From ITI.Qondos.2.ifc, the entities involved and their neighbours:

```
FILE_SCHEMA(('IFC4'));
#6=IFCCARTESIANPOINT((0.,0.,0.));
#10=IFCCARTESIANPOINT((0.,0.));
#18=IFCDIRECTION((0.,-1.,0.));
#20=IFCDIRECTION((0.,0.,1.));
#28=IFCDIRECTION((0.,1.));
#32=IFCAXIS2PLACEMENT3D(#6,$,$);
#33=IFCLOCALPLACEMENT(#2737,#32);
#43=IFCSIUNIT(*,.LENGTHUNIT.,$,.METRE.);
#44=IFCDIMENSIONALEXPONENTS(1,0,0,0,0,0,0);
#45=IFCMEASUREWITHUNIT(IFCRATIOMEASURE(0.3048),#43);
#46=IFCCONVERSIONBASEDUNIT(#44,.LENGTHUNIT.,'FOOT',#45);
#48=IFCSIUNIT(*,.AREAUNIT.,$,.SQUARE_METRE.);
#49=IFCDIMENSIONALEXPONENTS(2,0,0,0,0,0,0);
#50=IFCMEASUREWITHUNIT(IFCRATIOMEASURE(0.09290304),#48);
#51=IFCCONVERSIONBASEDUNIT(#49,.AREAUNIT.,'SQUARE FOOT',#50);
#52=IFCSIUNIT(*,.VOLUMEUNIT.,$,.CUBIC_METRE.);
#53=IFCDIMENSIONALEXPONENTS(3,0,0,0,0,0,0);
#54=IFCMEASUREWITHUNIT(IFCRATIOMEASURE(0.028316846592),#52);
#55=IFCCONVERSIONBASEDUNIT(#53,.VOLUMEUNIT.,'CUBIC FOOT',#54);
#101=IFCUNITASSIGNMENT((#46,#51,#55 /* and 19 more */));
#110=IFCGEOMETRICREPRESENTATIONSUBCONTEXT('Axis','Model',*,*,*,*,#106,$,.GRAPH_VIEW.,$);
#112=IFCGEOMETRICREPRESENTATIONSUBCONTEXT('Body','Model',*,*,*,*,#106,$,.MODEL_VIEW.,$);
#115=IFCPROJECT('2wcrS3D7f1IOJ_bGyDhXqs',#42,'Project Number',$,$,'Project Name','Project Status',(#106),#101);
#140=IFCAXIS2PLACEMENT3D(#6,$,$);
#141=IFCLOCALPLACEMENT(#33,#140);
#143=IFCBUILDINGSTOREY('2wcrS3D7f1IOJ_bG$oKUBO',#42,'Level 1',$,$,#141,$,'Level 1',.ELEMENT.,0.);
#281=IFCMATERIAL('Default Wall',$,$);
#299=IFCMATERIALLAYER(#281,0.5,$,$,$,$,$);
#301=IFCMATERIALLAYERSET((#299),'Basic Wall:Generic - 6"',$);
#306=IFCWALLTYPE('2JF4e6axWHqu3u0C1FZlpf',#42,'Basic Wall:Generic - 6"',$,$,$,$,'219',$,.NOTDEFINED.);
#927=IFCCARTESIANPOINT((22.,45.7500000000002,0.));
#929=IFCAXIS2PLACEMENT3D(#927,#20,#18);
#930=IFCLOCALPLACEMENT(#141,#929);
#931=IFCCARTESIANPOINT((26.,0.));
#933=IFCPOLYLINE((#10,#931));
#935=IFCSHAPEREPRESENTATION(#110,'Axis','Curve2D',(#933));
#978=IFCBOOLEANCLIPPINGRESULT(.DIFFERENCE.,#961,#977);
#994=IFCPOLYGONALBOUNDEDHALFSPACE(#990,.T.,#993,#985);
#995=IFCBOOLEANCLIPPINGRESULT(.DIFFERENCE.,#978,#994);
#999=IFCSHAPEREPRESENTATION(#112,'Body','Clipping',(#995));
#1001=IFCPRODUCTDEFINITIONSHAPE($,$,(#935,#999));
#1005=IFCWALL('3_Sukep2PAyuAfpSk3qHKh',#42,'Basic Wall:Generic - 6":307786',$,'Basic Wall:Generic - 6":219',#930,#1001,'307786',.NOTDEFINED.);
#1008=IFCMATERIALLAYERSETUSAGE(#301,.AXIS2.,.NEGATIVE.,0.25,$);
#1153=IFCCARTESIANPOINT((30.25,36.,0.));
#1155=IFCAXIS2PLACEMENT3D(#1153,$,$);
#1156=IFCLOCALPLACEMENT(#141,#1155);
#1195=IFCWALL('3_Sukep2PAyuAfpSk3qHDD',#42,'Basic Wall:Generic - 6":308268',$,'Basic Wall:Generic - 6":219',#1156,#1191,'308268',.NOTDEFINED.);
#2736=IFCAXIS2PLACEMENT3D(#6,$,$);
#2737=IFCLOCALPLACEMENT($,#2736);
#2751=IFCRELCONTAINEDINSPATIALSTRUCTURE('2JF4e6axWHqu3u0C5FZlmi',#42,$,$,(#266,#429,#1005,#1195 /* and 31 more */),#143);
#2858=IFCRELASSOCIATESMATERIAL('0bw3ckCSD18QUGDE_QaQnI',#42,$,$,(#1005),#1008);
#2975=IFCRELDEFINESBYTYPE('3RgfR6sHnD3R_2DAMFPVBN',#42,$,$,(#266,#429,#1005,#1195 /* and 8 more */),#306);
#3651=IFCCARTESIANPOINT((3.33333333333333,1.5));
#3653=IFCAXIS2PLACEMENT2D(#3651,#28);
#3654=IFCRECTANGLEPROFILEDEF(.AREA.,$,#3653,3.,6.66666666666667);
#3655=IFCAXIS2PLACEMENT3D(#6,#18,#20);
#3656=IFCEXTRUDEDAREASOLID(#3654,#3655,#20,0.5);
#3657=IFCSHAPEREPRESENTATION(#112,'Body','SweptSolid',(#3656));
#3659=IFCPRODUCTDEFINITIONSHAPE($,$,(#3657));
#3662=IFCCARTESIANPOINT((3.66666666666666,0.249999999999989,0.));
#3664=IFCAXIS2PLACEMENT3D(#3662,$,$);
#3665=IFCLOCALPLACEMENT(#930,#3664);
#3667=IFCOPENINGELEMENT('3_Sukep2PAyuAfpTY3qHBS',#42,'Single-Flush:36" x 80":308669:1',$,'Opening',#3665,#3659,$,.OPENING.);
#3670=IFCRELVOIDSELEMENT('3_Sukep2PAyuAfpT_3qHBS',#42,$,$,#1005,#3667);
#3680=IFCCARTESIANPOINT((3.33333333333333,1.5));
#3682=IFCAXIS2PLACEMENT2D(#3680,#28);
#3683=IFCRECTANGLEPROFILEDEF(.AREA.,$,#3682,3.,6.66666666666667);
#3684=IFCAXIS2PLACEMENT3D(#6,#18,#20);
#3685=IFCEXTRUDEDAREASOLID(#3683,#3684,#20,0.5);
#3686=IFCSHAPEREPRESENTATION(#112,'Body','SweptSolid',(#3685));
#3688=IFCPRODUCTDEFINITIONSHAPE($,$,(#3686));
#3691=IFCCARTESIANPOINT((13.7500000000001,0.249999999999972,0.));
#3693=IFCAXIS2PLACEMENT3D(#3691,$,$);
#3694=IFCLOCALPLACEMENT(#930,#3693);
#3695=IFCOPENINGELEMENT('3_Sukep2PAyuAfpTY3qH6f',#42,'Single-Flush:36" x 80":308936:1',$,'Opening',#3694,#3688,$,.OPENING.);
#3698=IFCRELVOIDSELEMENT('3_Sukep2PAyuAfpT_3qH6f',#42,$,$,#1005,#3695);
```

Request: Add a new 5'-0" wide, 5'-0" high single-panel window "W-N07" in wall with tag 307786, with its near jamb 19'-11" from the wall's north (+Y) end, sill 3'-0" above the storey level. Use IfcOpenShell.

```python
import numpy as np
import ifcopenshell
import ifcopenshell.api.feature
import ifcopenshell.api.geometry
import ifcopenshell.api.root
import ifcopenshell.api.spatial
import ifcopenshell.geom
import ifcopenshell.util.element
import ifcopenshell.util.placement
import ifcopenshell.util.representation
import ifcopenshell.util.shape
import ifcopenshell.util.unit

model = ifcopenshell.open("ITI.Qondos.2.ifc")
unit_scale = ifcopenshell.util.unit.calculate_unit_scale(model)
settings = ifcopenshell.geom.settings()


def volume(element):
    """Net volume in cubic metres, openings subtracted."""
    shape = ifcopenshell.geom.create_shape(settings, element)
    return ifcopenshell.util.shape.get_volume(shape.geometry)


wall = model.by_guid("3_Sukep2PAyuAfpSk3qHKh")
storey = ifcopenshell.util.element.get_container(wall, ifc_class="IfcBuildingStorey")
context = ifcopenshell.util.representation.get_context(model, "Model", "Body", "MODEL_VIEW")
before = volume(wall)

width, height, from_end, sill = 1.524, 1.524, 6.0706, 0.9144  # metres

# The wall runs along its own X axis, and the end named is its -X end.
wall_shape = ifcopenshell.geom.create_shape(settings, wall)
x, y, z = ifcopenshell.util.shape.get_vertices(wall_shape.geometry).T
start = x.min() + from_end
face, thickness = float(y.min()), float(y.max() - y.min())
wall_matrix = ifcopenshell.util.placement.get_local_placement(wall.ObjectPlacement)
level = ifcopenshell.util.placement.get_local_placement(storey.ObjectPlacement)[2, 3]


def in_wall(x, y):
    """Placement at x, y metres in the wall's axes, at sill height."""
    matrix = wall_matrix.copy()
    matrix[:, 3] = wall_matrix @ np.array([x / unit_scale, y / unit_scale, 0.0, 1.0])
    matrix[2, 3] = level + sill / unit_scale
    return matrix


# Opening: a box that overshoots both wall faces by 50 mm.
opening = ifcopenshell.api.root.create_entity(model, ifc_class="IfcOpeningElement", predefined_type="OPENING")
box = ifcopenshell.api.geometry.add_wall_representation(
    model, context=context, length=width, height=height, thickness=thickness + 0.1
)
ifcopenshell.api.geometry.assign_representation(model, product=opening, representation=box)
ifcopenshell.api.geometry.edit_object_placement(model, product=opening, matrix=in_wall(start, face - 0.05), is_si=False)
ifcopenshell.api.feature.add_feature(model, feature=opening, element=wall)

window = ifcopenshell.api.root.create_entity(model, ifc_class="IfcWindow", name="W-N07", predefined_type="WINDOW")
window.OverallWidth, window.OverallHeight = width / unit_scale, height / unit_scale
window.PartitioningType = "SINGLE_PANEL"
body = ifcopenshell.api.geometry.add_window_representation(
    model,
    context=context,
    overall_width=window.OverallWidth,
    overall_height=window.OverallHeight,
    partition_type="SINGLE_PANEL",
)
ifcopenshell.api.geometry.assign_representation(model, product=window, representation=body)
ifcopenshell.api.spatial.assign_container(model, products=[window], relating_structure=storey)
ifcopenshell.api.feature.add_filling(model, opening=opening, element=window)

# Centre the window in the wall's thickness.
ifcopenshell.api.geometry.edit_object_placement(model, product=window, matrix=in_wall(start, face), is_si=False)
window_shape = ifcopenshell.geom.create_shape(settings, window)
depth = ifcopenshell.util.shape.get_vertices(window_shape.geometry)[:, 1]
offset = face + thickness / 2 - (depth.min() + depth.max()) / 2
ifcopenshell.api.geometry.edit_object_placement(model, product=window, matrix=in_wall(start, offset), is_si=False)

after = volume(wall)

print(f"wall volume {before:.3f} -> {after:.3f} m3")

model.write("ITI.Qondos.2_v2.ifc")
```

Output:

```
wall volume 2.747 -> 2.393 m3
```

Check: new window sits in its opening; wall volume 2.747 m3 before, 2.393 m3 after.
